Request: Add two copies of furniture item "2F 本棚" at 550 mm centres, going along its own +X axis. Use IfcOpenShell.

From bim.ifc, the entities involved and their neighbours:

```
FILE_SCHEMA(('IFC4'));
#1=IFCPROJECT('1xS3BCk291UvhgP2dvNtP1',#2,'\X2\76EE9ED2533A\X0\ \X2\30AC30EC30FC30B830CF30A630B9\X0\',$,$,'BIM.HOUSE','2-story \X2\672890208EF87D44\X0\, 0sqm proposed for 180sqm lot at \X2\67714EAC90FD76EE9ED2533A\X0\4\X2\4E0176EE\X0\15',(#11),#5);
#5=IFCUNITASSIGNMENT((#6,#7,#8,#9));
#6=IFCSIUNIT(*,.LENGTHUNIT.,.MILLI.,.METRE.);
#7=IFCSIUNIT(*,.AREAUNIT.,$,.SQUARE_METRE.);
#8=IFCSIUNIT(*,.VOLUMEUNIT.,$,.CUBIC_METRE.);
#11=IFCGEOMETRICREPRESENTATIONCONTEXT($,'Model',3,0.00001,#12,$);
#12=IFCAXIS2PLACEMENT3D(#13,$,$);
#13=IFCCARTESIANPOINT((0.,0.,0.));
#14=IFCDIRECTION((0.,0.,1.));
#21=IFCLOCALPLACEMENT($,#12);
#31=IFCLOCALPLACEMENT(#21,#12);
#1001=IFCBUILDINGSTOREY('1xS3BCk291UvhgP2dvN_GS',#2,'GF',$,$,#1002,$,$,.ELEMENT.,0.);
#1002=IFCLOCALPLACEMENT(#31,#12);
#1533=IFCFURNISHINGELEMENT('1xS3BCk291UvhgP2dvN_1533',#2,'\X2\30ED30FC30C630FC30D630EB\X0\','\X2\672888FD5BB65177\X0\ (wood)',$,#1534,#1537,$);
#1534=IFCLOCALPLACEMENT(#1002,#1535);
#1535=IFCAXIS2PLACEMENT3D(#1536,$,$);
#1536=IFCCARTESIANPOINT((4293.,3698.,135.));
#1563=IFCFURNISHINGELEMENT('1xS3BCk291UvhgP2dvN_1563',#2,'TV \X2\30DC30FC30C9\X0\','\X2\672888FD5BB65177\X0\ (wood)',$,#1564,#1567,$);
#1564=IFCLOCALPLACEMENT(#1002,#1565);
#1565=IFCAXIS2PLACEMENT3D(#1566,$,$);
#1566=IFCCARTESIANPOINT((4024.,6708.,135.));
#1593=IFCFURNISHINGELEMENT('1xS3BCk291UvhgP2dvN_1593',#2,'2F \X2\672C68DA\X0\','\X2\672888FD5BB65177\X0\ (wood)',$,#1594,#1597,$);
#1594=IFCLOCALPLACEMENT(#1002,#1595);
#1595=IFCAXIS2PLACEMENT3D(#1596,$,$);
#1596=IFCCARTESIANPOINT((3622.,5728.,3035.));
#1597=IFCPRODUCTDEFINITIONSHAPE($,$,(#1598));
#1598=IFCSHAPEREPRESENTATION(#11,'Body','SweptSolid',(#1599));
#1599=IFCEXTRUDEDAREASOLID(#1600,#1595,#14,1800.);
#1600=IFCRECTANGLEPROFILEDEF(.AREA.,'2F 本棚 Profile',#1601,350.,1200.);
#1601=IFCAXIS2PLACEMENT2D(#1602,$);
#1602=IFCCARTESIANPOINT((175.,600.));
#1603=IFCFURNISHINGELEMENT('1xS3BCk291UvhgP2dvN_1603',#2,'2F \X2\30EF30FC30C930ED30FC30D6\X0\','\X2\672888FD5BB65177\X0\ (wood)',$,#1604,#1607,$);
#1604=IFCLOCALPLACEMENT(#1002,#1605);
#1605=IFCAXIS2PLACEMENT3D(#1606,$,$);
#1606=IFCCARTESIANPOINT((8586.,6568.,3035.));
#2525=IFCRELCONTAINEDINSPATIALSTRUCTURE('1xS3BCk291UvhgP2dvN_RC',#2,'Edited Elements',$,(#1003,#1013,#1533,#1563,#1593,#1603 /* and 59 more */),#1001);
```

```python
import ifcopenshell
import ifcopenshell.api.geometry
import ifcopenshell.api.root
import ifcopenshell.util.element
import ifcopenshell.util.placement

model = ifcopenshell.open("bim.ifc")


def reuse_history(source, copy):
    """copy_class also copies each property set's owner history, people and application; keep the originals."""
    for rel in copy.IsDefinedBy:
        if rel.is_a("IfcRelDefinesByProperties") and (history := rel.RelatingPropertyDefinition.OwnerHistory):
            rel.RelatingPropertyDefinition.OwnerHistory = source.OwnerHistory
            ifcopenshell.util.element.remove_deep2(model, history)


source = model.by_guid("1xS3BCk291UvhgP2dvN_1593")
base = ifcopenshell.util.placement.get_local_placement(source.ObjectPlacement)
step = base[:3, 0] * 550.0

for i in range(1, 3):
    copy = ifcopenshell.api.root.copy_class(model, product=source)
    copy.Representation = ifcopenshell.util.element.copy_deep(
        model, source.Representation, exclude=["IfcGeometricRepresentationContext", "IfcRepresentationMap"]
    )
    reuse_history(source, copy)
    matrix = base.copy()
    matrix[:3, 3] += i * step
    print("added at", matrix[:3, 3].round(3) + 0.0)
    ifcopenshell.api.geometry.edit_object_placement(model, product=copy, matrix=matrix, is_si=False)

model.write("bim_updated.ifc")
```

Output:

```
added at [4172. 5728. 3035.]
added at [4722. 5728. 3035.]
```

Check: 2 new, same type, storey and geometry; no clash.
